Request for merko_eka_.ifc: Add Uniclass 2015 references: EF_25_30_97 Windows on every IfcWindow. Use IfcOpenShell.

First a look at what the model holds.

```python
import ifcopenshell

model = ifcopenshell.open("merko_eka_.ifc")
print(model.schema)
print("classifications:", [c.Name for c in model.by_type("IfcClassification")])
for ifc_class in ("IfcDoor", "IfcRoof", "IfcStair", "IfcWall", "IfcWindow"):
    print(ifc_class, len(model.by_type(ifc_class)))
```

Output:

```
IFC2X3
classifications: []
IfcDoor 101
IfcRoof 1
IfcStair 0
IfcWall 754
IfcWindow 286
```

```python
import ifcopenshell
import ifcopenshell.api.classification

model = ifcopenshell.open("merko_eka_.ifc")

# IFC2X3 requires Source and Edition and has no link from the project to the system.
system = model.create_entity("IfcClassification", Source="NBS", Edition="2015", Name="Uniclass 2015")

codes = {
    "IfcWindow": ("EF_25_30_97", "Windows"),
}
for ifc_class, (code, name) in codes.items():
    products = model.by_type(ifc_class)
    ifcopenshell.api.classification.add_reference(
        model, products=products, classification=system, identification=code, name=name
    )
    print(code, len(products))

model.write("merko_eka_-out.ifc")
```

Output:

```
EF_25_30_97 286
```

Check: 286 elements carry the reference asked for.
